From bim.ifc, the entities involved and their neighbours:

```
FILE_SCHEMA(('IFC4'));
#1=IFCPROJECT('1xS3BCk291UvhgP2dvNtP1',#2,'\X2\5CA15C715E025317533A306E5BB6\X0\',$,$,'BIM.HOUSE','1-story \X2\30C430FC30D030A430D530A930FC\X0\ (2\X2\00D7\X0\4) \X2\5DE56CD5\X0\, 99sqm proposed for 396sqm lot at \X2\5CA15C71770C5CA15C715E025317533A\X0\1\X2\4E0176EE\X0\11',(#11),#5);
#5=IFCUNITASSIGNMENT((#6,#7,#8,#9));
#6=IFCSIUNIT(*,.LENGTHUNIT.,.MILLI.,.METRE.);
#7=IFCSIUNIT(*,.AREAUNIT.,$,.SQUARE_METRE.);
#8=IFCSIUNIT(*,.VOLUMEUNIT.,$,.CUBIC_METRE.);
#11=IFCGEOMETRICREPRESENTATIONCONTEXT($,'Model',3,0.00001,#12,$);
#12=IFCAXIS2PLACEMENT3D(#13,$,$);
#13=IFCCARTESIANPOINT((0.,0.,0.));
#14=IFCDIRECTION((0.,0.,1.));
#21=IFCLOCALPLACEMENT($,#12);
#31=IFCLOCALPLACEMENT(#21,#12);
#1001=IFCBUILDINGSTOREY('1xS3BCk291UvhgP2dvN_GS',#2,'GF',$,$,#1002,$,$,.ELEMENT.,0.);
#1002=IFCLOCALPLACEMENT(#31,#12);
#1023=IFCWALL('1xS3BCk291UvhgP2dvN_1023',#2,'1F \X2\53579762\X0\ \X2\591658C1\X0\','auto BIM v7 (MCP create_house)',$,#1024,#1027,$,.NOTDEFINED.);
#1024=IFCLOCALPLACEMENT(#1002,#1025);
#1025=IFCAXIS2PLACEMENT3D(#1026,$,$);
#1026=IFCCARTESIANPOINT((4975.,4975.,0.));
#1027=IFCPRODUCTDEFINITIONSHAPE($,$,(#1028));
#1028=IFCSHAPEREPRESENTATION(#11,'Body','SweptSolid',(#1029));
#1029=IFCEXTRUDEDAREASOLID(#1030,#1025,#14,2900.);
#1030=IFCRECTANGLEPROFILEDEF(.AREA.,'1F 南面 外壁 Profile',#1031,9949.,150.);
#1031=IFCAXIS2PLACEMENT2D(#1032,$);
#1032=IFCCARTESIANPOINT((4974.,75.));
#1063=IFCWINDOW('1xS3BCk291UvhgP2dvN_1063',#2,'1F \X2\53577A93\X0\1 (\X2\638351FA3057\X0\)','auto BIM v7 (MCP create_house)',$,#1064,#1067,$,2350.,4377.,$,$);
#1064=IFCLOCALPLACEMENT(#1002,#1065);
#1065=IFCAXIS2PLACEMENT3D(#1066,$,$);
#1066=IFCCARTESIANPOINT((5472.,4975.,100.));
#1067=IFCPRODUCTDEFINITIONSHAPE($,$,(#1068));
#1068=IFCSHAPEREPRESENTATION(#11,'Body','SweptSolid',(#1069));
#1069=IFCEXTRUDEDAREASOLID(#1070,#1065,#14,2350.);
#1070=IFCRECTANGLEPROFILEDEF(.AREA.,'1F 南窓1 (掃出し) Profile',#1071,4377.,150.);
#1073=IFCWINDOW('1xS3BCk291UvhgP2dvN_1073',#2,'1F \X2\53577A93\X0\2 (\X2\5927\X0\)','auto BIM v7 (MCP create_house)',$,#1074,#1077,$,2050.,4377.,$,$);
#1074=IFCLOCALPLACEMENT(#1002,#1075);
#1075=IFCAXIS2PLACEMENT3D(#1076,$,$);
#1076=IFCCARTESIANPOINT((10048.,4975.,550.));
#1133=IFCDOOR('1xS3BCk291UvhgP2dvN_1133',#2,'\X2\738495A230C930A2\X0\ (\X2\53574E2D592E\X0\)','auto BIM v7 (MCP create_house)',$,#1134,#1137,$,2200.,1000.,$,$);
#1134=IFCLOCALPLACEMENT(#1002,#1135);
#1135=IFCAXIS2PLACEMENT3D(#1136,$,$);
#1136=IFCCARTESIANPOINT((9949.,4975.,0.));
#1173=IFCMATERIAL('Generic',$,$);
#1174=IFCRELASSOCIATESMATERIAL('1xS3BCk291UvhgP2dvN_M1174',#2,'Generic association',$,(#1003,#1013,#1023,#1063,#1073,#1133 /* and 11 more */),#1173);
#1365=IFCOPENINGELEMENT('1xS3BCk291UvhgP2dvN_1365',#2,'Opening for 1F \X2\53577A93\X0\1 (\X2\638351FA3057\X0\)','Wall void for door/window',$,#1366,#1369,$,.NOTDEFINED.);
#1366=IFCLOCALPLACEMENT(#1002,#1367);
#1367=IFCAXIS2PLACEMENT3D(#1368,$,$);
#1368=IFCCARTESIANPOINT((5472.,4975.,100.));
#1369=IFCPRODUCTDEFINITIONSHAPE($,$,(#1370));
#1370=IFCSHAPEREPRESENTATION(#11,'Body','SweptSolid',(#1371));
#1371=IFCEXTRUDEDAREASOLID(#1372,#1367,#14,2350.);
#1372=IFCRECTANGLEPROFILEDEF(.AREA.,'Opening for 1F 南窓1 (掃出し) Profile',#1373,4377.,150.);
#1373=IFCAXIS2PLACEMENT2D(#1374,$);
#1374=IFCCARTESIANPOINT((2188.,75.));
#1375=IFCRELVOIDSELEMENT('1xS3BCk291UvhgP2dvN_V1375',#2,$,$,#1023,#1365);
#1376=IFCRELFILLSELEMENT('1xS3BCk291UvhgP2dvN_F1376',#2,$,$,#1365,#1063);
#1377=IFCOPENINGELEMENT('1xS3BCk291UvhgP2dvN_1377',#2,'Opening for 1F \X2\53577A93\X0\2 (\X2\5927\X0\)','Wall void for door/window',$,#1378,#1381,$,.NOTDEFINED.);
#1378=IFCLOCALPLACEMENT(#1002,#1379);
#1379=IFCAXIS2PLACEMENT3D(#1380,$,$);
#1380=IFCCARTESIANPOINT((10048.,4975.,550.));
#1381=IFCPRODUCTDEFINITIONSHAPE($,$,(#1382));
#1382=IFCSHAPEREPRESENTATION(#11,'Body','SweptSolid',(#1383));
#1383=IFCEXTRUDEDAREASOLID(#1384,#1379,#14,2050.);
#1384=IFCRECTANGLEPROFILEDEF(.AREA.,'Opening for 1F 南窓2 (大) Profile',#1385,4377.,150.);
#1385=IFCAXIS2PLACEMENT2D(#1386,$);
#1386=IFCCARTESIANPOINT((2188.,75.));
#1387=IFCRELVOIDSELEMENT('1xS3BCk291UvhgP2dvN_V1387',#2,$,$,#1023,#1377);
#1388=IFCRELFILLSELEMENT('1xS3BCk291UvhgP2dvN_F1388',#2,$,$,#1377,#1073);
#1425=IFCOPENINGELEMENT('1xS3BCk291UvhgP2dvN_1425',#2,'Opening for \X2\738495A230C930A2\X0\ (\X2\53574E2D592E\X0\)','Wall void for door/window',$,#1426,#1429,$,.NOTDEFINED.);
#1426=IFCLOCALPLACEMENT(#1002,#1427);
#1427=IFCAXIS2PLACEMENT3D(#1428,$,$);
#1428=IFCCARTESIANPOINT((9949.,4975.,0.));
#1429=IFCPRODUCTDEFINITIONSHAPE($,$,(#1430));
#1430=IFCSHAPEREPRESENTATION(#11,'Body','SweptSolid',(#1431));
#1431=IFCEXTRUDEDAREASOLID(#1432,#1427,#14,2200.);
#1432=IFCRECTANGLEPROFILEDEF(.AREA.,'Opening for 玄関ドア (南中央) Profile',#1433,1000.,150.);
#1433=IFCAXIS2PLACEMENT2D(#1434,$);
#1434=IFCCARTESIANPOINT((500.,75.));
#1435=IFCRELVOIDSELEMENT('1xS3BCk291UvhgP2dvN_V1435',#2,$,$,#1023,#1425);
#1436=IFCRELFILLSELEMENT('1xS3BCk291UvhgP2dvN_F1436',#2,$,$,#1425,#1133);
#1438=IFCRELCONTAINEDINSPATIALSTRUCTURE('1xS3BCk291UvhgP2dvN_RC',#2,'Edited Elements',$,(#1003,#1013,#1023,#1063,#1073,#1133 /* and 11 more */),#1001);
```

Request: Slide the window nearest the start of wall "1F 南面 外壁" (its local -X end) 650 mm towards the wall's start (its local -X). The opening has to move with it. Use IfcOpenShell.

```python
import ifcopenshell
import ifcopenshell.api.geometry
import ifcopenshell.util.placement
import ifcopenshell.util.unit

model = ifcopenshell.open("bim.ifc")
unit_scale = ifcopenshell.util.unit.calculate_unit_scale(model)

window = model.by_guid("1xS3BCk291UvhgP2dvN_1063")
opening = window.FillsVoids[0].RelatingOpeningElement
wall = opening.VoidsElements[0].RelatingBuildingElement

wall_matrix = ifcopenshell.util.placement.get_local_placement(wall.ObjectPlacement)
shift = wall_matrix[:3, 0] * -0.65 / unit_scale
before = ifcopenshell.util.placement.get_local_placement(window.ObjectPlacement)[:3, 3].copy()

# The window is not placed relative to its opening, so move both.
for product in (opening, window):
    matrix = ifcopenshell.util.placement.get_local_placement(product.ObjectPlacement)
    matrix[:3, 3] += shift
    ifcopenshell.api.geometry.edit_object_placement(model, product=product, matrix=matrix, is_si=False)

after = ifcopenshell.util.placement.get_local_placement(window.ObjectPlacement)[:3, 3]
print("window moved by", (after - before).round(3) + 0.0)

model.write("bim_edited.ifc")
```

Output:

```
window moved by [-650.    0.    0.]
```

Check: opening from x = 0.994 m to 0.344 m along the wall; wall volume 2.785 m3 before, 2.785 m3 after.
